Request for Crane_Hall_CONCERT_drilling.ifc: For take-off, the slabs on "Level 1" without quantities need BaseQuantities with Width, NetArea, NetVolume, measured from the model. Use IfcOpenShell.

First a look at what the model holds.

```python
import ifcopenshell
import ifcopenshell.util.element
import ifcopenshell.util.unit

model = ifcopenshell.open("Crane_Hall_CONCERT_drilling.ifc")
print(model.schema)
for unit_type in ("LENGTHUNIT", "AREAUNIT", "VOLUMEUNIT"):
    print(unit_type, ifcopenshell.util.unit.calculate_unit_scale(model, unit_type))
storey = next(s for s in model.by_type("IfcBuildingStorey") if s.Name == "Level 1")
slabs = [e for e in ifcopenshell.util.element.get_decomposition(storey) if e.is_a("IfcSlab")]
for e in sorted(slabs, key=lambda e: e.id()):
    print(e.id(), e.is_a(), e.Name, list(ifcopenshell.util.element.get_psets(e, qtos_only=True)), sep=" | ")
```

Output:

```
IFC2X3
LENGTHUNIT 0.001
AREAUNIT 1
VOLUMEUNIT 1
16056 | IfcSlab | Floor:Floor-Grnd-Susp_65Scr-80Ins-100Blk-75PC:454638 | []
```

```python
import ifcopenshell
import ifcopenshell.api.pset
import ifcopenshell.geom
import ifcopenshell.util.element
import ifcopenshell.util.shape
import ifcopenshell.util.unit

model = ifcopenshell.open("Crane_Hall_CONCERT_drilling.ifc")
unit_scale = ifcopenshell.util.unit.calculate_unit_scale(model)
area_scale = ifcopenshell.util.unit.calculate_unit_scale(model, "AREAUNIT")
volume_scale = ifcopenshell.util.unit.calculate_unit_scale(model, "VOLUMEUNIT")
settings = ifcopenshell.geom.settings()

storey = next(s for s in model.by_type("IfcBuildingStorey") if s.Name == "Level 1")
slabs = [e for e in ifcopenshell.util.element.get_decomposition(storey) if e.is_a("IfcSlab")]

for e in sorted(slabs, key=lambda e: e.id()):
    if ifcopenshell.util.element.get_psets(e, qtos_only=True, should_inherit=False):
        continue
    # Geometry comes back in metres, in the element's own axes.
    shape = ifcopenshell.geom.create_shape(settings, e)
    values = {
        "Width": ifcopenshell.util.shape.get_z(shape.geometry) / unit_scale,
        "NetArea": ifcopenshell.util.shape.get_footprint_area(shape.geometry) / area_scale,
        "NetVolume": ifcopenshell.util.shape.get_volume(shape.geometry) / volume_scale,
    }
    qto = ifcopenshell.api.pset.add_qto(model, product=e, name="BaseQuantities")
    ifcopenshell.api.pset.edit_qto(model, qto=qto, properties=values)
    print(e.id(), {k: round(v, 3) for k, v in values.items()})

model.write("Crane_Hall_CONCERT_drilling_rev.ifc")
```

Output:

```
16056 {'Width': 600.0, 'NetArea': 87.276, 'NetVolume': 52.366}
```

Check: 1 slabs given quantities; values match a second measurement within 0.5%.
